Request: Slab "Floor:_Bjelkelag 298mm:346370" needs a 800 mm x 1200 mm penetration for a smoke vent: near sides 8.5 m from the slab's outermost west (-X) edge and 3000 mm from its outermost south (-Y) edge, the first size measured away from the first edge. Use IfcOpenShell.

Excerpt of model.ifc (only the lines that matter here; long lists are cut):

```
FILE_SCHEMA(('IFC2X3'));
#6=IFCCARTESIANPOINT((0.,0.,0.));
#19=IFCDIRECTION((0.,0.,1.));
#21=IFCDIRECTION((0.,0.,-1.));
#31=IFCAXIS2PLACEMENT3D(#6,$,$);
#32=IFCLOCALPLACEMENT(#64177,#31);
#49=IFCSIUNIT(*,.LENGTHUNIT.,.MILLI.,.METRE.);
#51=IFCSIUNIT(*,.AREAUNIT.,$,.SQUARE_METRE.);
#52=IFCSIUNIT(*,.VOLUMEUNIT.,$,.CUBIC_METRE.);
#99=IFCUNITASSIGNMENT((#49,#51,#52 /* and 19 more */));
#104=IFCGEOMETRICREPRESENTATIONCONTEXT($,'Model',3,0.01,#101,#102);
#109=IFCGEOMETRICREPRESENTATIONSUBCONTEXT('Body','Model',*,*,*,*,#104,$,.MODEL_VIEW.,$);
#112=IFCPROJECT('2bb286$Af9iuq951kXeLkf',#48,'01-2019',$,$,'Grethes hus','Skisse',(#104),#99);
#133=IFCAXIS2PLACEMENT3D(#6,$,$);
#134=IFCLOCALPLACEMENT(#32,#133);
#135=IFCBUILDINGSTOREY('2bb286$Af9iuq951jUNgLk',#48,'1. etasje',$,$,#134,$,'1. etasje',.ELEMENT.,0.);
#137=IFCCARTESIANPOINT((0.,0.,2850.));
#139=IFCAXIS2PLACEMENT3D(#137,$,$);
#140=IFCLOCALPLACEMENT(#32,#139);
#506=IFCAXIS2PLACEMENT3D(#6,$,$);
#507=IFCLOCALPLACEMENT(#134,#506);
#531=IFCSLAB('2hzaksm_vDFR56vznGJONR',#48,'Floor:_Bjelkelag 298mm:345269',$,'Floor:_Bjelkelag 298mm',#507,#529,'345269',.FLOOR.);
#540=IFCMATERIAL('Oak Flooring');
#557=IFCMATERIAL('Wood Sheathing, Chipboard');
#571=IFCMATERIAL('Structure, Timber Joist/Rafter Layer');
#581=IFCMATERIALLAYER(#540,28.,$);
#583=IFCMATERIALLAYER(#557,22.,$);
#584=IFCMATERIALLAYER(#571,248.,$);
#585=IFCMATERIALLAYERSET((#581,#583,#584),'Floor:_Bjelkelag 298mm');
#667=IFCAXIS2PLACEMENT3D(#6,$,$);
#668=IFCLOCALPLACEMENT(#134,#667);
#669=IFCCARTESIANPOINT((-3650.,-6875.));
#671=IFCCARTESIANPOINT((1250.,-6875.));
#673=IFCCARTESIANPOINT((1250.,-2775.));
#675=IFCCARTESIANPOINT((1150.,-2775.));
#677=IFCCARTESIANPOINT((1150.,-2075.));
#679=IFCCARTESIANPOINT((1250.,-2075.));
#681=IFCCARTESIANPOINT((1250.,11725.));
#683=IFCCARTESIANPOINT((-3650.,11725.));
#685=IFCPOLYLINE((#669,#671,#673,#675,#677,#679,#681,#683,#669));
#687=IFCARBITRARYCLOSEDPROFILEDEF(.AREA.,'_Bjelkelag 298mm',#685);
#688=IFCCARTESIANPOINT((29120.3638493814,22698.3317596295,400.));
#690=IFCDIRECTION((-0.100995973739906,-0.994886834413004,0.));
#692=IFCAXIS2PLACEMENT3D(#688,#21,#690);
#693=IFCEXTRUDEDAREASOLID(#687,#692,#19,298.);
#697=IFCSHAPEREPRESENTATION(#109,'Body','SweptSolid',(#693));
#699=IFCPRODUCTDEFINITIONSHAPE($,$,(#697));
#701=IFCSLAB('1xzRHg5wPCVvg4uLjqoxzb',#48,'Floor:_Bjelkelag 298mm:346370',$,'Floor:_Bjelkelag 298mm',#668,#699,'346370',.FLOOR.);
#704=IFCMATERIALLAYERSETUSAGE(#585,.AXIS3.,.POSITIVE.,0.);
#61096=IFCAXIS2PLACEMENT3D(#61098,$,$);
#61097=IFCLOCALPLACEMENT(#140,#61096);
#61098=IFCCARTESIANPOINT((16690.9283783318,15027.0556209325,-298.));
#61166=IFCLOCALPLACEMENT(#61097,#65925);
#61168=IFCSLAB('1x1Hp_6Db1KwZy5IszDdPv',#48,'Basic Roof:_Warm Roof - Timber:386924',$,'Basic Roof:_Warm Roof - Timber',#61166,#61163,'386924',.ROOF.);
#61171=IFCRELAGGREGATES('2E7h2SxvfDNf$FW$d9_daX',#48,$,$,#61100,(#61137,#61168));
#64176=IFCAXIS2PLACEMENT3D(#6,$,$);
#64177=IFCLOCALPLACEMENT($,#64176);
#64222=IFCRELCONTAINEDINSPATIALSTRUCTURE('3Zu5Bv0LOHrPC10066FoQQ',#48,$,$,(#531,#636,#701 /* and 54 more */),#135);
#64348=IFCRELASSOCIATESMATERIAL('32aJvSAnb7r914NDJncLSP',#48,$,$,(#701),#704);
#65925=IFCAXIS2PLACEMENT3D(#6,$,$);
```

```python
import numpy as np
import ifcopenshell
import ifcopenshell.api.feature
import ifcopenshell.api.geometry
import ifcopenshell.api.root
import ifcopenshell.geom
import ifcopenshell.util.placement
import ifcopenshell.util.representation
import ifcopenshell.util.shape
import ifcopenshell.util.unit

model = ifcopenshell.open("model.ifc")
unit_scale = ifcopenshell.util.unit.calculate_unit_scale(model)
settings = ifcopenshell.geom.settings()


def volume(element):
    """Net volume in cubic metres, openings subtracted."""
    shape = ifcopenshell.geom.create_shape(settings, element)
    return ifcopenshell.util.shape.get_volume(shape.geometry)


slab = model.by_id(701)
before = volume(slab)

# Extent in the slab's own axes, in metres. The edges named are its -X and -Y sides.
slab_shape = ifcopenshell.geom.create_shape(settings, slab)
vertices = ifcopenshell.util.shape.get_vertices(slab_shape.geometry)
x_min, y_min, bottom = vertices.min(axis=0)
top = vertices[:, 2].max()

opening = ifcopenshell.api.root.create_entity(model, ifc_class="IfcOpeningElement", name="Smoke vent opening")
context = ifcopenshell.util.representation.get_context(model, "Model", "Body", "MODEL_VIEW")
width, depth = 0.8, 1.2
outline = [(0.0, 0.0), (width, 0.0), (width, depth), (0.0, depth), (0.0, 0.0)]
# Overshoot both faces by 50 mm so the cut is clean.
shape = ifcopenshell.api.geometry.add_slab_representation(
    model, context=context, depth=top - bottom + 0.1, polyline=outline
)
ifcopenshell.api.geometry.assign_representation(model, product=opening, representation=shape)

matrix = ifcopenshell.util.placement.get_local_placement(slab.ObjectPlacement)
matrix[:, 3] = matrix @ np.append(np.array([x_min + 8.5, y_min + 3, bottom - 0.05]) / unit_scale, 1.0)
ifcopenshell.api.geometry.edit_object_placement(model, product=opening, matrix=matrix, is_si=False)
ifcopenshell.api.feature.add_feature(model, feature=opening, element=slab)

after = volume(slab)

print(f"slab volume {before:.3f} -> {after:.3f} m3")

model.write("model_rev.ifc")
```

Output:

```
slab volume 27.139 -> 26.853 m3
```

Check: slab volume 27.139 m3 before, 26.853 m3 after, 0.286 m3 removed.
